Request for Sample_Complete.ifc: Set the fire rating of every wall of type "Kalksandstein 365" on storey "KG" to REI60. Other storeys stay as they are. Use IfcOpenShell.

First a look at what the model holds.

```python
import ifcopenshell
import ifcopenshell.util.element

model = ifcopenshell.open("Sample_Complete.ifc")
print(model.schema)
storey = next(s for s in model.by_type("IfcBuildingStorey") if s.Name == "KG")
walls = [e for e in ifcopenshell.util.element.get_decomposition(storey) if e.is_a("IfcWall")]
seen = {}
for e in walls:
    element_type = ifcopenshell.util.element.get_type(e)
    key = (element_type.Name if element_type != e and element_type else None, ifcopenshell.util.element.get_pset(e, "Pset_WallCommon", "FireRating"))
    seen[key] = seen.get(key, 0) + 1
for (name, value), count in sorted(seen.items(), key=str):
    print(count, "x", name, "|", value)
```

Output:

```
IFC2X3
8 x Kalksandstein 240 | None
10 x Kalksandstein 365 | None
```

```python
import ifcopenshell
import ifcopenshell.api.pset
import ifcopenshell.util.element

model = ifcopenshell.open("Sample_Complete.ifc")

storey = next(s for s in model.by_type("IfcBuildingStorey") if s.Name == "KG")
walls = [e for e in ifcopenshell.util.element.get_decomposition(storey) if e.is_a("IfcWall")]

count = 0
for e in walls:
    element_type = ifcopenshell.util.element.get_type(e)
    if element_type in (None, e) or element_type.Name != "Kalksandstein 365":
        continue
    # add_pset returns the element's existing set when there is one.
    pset = ifcopenshell.api.pset.add_pset(model, product=e, name="Pset_WallCommon")
    ifcopenshell.api.pset.edit_pset(model, pset=pset, properties={"FireRating": "REI60"})
    count += 1

print(count, "walls updated")

model.write("Sample_Complete_edited.ifc")
```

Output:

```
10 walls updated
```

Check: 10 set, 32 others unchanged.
